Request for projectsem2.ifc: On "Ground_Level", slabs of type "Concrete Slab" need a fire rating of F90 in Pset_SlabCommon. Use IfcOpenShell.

First a look at what the model holds.

```python
import ifcopenshell
import ifcopenshell.util.element

model = ifcopenshell.open("projectsem2.ifc")
print(model.schema)
storey = next(s for s in model.by_type("IfcBuildingStorey") if s.Name == "Ground_Level")
slabs = [e for e in ifcopenshell.util.element.get_decomposition(storey) if e.is_a("IfcSlab")]
seen = {}
for e in slabs:
    element_type = ifcopenshell.util.element.get_type(e)
    key = (element_type.Name if element_type != e and element_type else None, ifcopenshell.util.element.get_pset(e, "Pset_SlabCommon", "FireRating"))
    seen[key] = seen.get(key, 0) + 1
for (name, value), count in sorted(seen.items(), key=str):
    print(count, "x", name, "|", value)
```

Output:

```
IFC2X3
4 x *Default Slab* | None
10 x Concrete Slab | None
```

```python
import ifcopenshell
import ifcopenshell.api.pset
import ifcopenshell.util.element

model = ifcopenshell.open("projectsem2.ifc")

storey = next(s for s in model.by_type("IfcBuildingStorey") if s.Name == "Ground_Level")
slabs = [e for e in ifcopenshell.util.element.get_decomposition(storey) if e.is_a("IfcSlab")]

count = 0
for e in slabs:
    element_type = ifcopenshell.util.element.get_type(e)
    if element_type in (None, e) or element_type.Name != "Concrete Slab":
        continue
    # add_pset returns the element's existing set when there is one.
    pset = ifcopenshell.api.pset.add_pset(model, product=e, name="Pset_SlabCommon")
    ifcopenshell.api.pset.edit_pset(model, pset=pset, properties={"FireRating": "F90"})
    count += 1

print(count, "slabs updated")

model.write("projectsem2_rev.ifc")
```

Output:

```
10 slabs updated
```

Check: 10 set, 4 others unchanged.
